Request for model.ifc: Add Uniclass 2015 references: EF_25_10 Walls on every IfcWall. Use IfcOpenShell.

First a look at what the model holds.

```python
import ifcopenshell

model = ifcopenshell.open("model.ifc")
print(model.schema)
print("classifications:", [c.Name for c in model.by_type("IfcClassification")])
for ifc_class in ("IfcDoor", "IfcRoof", "IfcStair", "IfcWall", "IfcWindow"):
    print(ifc_class, len(model.by_type(ifc_class)))
```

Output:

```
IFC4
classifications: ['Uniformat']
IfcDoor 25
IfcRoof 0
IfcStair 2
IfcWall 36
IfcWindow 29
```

```python
import ifcopenshell
import ifcopenshell.api.classification

model = ifcopenshell.open("model.ifc")

system = ifcopenshell.api.classification.add_classification(model, classification="Uniclass 2015")

codes = {
    "IfcWall": ("EF_25_10", "Walls"),
}
for ifc_class, (code, name) in codes.items():
    products = model.by_type(ifc_class)
    ifcopenshell.api.classification.add_reference(
        model, products=products, classification=system, identification=code, name=name
    )
    print(code, len(products))

model.write("model_updated.ifc")
```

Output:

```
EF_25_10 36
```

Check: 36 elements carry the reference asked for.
